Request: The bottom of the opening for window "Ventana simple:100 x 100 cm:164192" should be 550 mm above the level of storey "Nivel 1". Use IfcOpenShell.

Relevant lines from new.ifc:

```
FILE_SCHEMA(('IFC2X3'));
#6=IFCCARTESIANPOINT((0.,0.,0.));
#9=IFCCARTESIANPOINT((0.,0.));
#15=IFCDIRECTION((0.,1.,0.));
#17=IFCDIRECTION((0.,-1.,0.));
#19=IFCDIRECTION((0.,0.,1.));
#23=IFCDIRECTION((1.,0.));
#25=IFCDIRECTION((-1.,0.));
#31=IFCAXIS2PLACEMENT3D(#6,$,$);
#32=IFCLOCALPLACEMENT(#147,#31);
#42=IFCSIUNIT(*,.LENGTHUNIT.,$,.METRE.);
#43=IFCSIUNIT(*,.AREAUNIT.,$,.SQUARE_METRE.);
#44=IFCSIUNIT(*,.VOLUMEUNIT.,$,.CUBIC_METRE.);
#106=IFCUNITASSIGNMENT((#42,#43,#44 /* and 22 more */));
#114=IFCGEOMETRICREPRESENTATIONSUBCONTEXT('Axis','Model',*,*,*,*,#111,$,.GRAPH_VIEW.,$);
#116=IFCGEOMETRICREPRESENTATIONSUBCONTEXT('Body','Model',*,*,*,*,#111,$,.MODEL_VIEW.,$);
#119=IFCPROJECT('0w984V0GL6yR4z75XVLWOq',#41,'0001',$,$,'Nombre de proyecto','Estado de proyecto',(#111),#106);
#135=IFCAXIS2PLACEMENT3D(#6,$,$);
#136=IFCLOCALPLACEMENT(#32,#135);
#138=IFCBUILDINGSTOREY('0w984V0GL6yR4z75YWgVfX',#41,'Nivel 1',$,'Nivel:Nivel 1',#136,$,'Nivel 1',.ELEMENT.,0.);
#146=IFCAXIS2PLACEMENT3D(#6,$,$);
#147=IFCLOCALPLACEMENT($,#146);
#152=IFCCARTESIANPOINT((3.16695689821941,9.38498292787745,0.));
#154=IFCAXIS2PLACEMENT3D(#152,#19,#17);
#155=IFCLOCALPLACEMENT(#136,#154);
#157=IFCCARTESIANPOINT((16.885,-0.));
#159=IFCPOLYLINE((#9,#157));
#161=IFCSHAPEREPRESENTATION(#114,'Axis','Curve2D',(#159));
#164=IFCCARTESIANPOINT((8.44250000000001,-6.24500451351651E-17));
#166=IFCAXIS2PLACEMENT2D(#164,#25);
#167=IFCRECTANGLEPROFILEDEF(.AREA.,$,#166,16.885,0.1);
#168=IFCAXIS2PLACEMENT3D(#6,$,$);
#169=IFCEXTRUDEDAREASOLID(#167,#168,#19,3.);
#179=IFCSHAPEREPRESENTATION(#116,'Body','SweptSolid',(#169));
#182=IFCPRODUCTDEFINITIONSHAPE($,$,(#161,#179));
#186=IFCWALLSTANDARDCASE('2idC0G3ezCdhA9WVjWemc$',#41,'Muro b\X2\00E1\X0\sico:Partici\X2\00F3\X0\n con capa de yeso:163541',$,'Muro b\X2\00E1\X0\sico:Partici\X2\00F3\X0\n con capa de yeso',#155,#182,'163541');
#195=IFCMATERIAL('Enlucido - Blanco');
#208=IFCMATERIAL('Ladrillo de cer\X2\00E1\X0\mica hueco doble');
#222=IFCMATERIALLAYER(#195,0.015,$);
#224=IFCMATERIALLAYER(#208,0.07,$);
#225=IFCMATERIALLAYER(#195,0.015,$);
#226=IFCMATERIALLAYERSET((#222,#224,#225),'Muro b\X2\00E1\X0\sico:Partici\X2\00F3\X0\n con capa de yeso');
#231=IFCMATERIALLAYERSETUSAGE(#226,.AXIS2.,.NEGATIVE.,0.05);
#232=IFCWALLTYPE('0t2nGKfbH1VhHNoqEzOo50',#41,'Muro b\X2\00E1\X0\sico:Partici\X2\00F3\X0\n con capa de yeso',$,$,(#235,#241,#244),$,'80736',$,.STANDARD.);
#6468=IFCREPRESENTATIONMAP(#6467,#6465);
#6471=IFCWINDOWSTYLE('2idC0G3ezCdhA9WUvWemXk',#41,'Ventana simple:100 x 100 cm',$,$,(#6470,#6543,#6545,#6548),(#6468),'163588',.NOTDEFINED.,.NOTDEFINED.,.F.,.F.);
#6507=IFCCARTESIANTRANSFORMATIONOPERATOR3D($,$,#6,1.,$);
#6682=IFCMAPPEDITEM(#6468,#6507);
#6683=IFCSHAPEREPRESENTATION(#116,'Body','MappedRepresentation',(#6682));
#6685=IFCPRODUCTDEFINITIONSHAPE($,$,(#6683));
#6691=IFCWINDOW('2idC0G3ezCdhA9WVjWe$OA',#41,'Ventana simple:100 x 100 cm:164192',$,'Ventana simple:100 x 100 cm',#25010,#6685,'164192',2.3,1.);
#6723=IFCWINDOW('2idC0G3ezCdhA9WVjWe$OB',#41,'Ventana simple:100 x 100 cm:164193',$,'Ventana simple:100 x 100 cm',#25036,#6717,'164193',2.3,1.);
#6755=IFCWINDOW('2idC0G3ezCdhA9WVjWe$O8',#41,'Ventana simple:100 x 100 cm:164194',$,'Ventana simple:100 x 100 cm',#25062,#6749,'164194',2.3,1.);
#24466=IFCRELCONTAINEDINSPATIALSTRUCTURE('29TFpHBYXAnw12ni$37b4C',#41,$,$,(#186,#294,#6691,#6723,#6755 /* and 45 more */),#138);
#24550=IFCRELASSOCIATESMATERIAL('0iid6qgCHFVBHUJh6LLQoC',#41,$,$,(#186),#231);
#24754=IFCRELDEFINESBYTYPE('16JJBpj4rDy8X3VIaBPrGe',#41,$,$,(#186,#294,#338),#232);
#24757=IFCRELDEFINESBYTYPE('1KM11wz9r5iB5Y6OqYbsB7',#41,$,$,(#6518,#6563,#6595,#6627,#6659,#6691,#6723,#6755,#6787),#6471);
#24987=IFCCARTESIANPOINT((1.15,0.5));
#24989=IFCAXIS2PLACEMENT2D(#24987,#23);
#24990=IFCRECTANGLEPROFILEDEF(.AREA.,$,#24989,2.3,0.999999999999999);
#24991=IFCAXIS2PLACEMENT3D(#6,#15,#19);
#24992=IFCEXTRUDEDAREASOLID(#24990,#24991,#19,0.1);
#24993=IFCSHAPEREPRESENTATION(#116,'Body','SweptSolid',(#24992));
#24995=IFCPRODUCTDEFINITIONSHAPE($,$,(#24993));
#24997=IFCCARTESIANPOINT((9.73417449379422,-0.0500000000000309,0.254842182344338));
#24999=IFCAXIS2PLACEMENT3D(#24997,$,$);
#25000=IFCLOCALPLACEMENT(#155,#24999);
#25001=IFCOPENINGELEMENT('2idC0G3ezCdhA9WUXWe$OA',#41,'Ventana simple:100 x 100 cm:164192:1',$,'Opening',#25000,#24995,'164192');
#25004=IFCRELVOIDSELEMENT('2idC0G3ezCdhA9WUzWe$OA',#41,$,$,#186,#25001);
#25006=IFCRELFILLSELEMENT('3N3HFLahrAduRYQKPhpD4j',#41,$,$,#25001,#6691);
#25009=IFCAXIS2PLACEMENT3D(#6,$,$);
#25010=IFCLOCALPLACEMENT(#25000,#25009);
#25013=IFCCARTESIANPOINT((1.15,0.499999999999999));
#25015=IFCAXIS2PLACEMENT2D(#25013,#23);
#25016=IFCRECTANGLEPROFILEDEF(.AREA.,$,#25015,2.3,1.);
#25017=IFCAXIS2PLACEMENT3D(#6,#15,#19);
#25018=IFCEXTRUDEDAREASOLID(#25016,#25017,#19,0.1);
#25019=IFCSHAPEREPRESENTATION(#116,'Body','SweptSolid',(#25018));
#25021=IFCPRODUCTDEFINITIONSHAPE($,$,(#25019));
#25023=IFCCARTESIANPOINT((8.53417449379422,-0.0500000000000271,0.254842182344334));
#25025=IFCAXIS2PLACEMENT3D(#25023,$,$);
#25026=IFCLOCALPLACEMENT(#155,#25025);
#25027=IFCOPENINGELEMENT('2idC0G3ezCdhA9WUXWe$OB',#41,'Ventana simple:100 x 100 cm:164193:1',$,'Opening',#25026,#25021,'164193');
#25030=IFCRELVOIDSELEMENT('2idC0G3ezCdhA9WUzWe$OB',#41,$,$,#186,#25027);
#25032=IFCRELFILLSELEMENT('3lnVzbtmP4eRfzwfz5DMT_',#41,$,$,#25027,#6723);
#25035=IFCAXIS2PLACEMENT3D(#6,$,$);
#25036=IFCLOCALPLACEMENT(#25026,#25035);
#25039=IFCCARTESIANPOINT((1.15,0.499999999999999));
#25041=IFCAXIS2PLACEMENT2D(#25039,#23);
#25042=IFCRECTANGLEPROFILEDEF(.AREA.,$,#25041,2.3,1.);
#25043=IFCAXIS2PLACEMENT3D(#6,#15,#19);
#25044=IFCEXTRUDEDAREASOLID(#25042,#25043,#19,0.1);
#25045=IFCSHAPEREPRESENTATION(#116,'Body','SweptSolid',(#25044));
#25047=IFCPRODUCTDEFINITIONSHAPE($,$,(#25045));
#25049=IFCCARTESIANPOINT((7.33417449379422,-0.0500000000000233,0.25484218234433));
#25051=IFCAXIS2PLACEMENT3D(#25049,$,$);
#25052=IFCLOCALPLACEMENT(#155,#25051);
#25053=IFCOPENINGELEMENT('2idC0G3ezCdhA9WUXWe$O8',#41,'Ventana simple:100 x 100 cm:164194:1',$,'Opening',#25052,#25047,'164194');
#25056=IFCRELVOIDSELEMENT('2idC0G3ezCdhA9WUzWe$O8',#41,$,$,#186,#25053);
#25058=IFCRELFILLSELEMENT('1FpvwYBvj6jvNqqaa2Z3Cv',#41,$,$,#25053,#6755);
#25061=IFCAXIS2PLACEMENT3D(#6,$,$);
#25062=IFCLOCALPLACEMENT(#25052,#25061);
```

```python
import numpy as np
import ifcopenshell
import ifcopenshell.api.geometry
import ifcopenshell.geom
import ifcopenshell.util.element
import ifcopenshell.util.placement
import ifcopenshell.util.shape
import ifcopenshell.util.unit

model = ifcopenshell.open("new.ifc")
unit_scale = ifcopenshell.util.unit.calculate_unit_scale(model)

window = model.by_id(6691)
opening = window.FillsVoids[0].RelatingOpeningElement
storey = ifcopenshell.util.element.get_container(window, ifc_class="IfcBuildingStorey")
level = ifcopenshell.util.placement.get_local_placement(storey.ObjectPlacement)[2, 3]

# The opening's origin need not be at the sill, so measure its lowest point.
shape = ifcopenshell.geom.create_shape(ifcopenshell.geom.settings(), opening)
bottom = ifcopenshell.util.shape.get_shape_bottom_elevation(shape, shape.geometry) / unit_scale
dz = level + 0.55 - bottom

shift = np.array([0.0, 0.0, dz])
# The window is placed relative to its opening, so it follows when the opening moves.
matrix = ifcopenshell.util.placement.get_local_placement(opening.ObjectPlacement)
matrix[:3, 3] += shift
ifcopenshell.api.geometry.edit_object_placement(
    model, product=opening, matrix=matrix, is_si=False, should_transform_children=True
)

print(f"moved by {dz * unit_scale:+.3f} m")

model.write("new-out.ifc")
```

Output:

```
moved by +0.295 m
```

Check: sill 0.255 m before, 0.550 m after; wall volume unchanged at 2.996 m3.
